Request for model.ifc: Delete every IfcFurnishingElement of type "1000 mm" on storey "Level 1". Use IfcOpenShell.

First a look at what the model holds.

```python
import ifcopenshell
import ifcopenshell.util.element

model = ifcopenshell.open("model.ifc")
print(model.schema)
storey = next(s for s in model.by_type("IfcBuildingStorey") if s.Name == "Level 1")
furniture = [e for e in ifcopenshell.util.element.get_decomposition(storey) if e.is_a("IfcFurnishingElement")]
seen = {}
for e in furniture:
    element_type = ifcopenshell.util.element.get_type(e)
    name = element_type.Name if element_type not in (None, e) else None
    seen[name] = seen.get(name, 0) + 1
for name, count in sorted(seen.items(), key=str):
    print(count, "x", name)
```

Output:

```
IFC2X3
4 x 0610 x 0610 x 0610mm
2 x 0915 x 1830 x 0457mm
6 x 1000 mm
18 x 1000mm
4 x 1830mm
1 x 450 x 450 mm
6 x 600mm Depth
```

```python
import ifcopenshell
import ifcopenshell.api.root
import ifcopenshell.util.element

model = ifcopenshell.open("model.ifc")

storey = next(s for s in model.by_type("IfcBuildingStorey") if s.Name == "Level 1")
furniture = [e for e in ifcopenshell.util.element.get_decomposition(storey) if e.is_a("IfcFurnishingElement")]
targets = [e for e in furniture if (t := ifcopenshell.util.element.get_type(e)) not in (None, e) and t.Name == "1000 mm"]

for e in targets:
    ifcopenshell.api.root.remove_product(model, product=e)
print(len(targets), "removed")

model.write("model_rev.ifc")
```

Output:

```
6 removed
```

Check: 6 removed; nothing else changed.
